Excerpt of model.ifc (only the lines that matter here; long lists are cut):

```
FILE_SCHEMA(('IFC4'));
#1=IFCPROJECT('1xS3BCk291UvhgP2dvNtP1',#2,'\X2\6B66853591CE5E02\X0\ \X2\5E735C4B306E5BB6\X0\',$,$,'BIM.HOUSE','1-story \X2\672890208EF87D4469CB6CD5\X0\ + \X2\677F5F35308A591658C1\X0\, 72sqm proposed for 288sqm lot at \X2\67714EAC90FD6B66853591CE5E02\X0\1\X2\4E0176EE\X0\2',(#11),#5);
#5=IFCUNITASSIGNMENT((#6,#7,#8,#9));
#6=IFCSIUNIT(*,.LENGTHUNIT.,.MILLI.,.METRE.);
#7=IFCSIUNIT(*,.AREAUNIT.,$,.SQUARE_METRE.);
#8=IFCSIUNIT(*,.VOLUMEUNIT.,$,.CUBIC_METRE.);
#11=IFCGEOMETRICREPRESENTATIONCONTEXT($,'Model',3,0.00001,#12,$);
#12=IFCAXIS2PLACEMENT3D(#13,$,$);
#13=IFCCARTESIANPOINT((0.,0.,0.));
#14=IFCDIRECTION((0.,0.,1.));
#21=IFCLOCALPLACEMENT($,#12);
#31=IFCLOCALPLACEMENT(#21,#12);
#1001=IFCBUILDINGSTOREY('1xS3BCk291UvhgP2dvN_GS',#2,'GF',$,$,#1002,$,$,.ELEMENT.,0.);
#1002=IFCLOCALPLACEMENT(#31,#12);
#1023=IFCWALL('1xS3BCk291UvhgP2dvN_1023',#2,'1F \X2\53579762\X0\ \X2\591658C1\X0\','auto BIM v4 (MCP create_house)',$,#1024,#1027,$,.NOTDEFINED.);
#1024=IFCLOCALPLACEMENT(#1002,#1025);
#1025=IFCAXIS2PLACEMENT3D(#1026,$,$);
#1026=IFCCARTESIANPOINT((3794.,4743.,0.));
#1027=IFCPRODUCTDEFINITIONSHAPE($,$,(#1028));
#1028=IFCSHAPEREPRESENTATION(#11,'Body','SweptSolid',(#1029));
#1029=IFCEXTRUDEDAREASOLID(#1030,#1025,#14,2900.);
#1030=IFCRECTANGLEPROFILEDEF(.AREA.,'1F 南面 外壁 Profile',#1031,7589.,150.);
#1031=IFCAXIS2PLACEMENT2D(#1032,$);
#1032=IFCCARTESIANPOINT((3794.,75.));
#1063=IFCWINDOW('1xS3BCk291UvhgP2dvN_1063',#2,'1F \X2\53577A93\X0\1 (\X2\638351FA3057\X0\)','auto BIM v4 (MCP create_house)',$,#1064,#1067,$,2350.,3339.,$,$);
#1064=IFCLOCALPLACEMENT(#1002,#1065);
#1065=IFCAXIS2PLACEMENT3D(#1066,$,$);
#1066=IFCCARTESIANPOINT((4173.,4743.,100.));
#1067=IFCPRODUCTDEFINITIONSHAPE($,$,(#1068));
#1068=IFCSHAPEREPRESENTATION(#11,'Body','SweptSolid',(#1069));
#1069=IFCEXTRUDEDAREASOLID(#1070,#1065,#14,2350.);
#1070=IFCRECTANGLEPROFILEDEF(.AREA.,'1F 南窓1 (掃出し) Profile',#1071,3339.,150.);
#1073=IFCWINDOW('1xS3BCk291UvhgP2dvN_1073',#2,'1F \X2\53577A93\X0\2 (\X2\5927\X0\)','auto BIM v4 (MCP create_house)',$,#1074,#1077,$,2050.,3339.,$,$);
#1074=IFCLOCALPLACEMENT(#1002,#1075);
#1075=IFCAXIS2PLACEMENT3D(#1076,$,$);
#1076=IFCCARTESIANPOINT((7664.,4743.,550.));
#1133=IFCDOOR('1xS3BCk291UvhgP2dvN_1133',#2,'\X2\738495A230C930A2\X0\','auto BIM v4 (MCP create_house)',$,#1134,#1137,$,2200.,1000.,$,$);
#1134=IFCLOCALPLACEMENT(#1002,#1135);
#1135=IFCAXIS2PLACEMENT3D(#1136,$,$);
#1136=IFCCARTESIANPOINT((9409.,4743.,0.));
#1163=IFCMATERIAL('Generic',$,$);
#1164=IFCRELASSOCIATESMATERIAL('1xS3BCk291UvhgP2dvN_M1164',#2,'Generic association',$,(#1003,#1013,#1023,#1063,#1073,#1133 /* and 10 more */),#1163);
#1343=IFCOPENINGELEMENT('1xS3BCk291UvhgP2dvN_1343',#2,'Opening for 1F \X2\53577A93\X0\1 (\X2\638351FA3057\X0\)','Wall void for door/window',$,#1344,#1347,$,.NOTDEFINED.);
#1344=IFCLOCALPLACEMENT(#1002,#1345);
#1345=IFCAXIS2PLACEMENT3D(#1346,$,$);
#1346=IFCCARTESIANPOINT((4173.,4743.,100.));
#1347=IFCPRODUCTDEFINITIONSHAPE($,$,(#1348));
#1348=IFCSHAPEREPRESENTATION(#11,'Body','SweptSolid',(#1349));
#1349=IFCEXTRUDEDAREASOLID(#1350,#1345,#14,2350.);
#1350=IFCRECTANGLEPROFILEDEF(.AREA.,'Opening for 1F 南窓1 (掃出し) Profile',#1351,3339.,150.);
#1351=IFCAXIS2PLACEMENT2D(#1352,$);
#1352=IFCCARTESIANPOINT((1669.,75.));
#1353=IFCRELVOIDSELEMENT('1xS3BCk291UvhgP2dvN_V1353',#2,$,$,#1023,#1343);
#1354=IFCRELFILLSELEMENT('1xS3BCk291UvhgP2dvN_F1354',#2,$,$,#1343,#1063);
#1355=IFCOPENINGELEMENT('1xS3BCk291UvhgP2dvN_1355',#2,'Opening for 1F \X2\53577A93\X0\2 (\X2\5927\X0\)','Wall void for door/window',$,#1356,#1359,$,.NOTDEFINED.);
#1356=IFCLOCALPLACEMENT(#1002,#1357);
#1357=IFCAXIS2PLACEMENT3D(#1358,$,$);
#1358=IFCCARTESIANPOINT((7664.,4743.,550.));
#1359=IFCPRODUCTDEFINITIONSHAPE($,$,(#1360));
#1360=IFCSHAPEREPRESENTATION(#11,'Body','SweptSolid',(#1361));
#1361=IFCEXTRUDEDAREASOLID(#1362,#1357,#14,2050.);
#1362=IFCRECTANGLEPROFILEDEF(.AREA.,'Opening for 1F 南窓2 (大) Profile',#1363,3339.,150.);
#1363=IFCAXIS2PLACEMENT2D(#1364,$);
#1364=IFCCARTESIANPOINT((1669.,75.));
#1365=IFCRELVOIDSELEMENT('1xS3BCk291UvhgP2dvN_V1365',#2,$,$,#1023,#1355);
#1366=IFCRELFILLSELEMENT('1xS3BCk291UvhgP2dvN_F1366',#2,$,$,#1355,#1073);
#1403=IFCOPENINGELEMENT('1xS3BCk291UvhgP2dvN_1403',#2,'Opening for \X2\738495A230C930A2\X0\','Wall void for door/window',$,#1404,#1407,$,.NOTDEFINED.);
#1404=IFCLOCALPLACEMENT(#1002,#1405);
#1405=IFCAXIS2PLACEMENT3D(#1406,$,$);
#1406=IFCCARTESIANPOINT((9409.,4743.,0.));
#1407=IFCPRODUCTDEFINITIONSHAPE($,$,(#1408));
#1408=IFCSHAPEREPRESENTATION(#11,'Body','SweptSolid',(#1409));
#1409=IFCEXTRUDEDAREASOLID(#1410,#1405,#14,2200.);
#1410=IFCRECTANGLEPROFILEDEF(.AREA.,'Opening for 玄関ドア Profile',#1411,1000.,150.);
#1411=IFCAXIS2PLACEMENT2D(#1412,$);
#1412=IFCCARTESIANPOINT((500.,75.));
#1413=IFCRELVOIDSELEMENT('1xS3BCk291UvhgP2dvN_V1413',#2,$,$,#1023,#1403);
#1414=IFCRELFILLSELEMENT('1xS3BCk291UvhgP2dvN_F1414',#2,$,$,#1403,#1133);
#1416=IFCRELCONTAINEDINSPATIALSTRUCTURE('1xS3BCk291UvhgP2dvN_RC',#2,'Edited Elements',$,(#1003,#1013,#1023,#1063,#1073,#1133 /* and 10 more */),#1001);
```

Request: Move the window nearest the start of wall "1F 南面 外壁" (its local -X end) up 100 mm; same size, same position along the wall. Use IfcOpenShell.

```python
import numpy as np
import ifcopenshell
import ifcopenshell.api.geometry
import ifcopenshell.util.placement
import ifcopenshell.util.unit

model = ifcopenshell.open("model.ifc")
unit_scale = ifcopenshell.util.unit.calculate_unit_scale(model)

window = model.by_id(1063)
opening = window.FillsVoids[0].RelatingOpeningElement
dz = 0.1 / unit_scale

shift = np.array([0.0, 0.0, dz])
# The window is not placed relative to its opening, so move both.
for product in (opening, window):
    matrix = ifcopenshell.util.placement.get_local_placement(product.ObjectPlacement)
    matrix[:3, 3] += shift
    ifcopenshell.api.geometry.edit_object_placement(model, product=product, matrix=matrix, is_si=False)

print(f"moved by {dz * unit_scale:+.3f} m")

model.write("model_v2.ifc")
```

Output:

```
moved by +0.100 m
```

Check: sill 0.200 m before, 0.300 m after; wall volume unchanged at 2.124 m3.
